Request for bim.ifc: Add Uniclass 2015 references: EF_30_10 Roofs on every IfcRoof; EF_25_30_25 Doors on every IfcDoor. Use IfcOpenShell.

First a look at what the model holds.

```python
import ifcopenshell

model = ifcopenshell.open("bim.ifc")
print(model.schema)
print("classifications:", [c.Name for c in model.by_type("IfcClassification")])
for ifc_class in ("IfcDoor", "IfcRoof", "IfcStair", "IfcWall", "IfcWindow"):
    print(ifc_class, len(model.by_type(ifc_class)))
```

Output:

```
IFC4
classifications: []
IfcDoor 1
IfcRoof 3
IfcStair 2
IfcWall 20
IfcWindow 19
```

```python
import ifcopenshell
import ifcopenshell.api.classification

model = ifcopenshell.open("bim.ifc")

system = ifcopenshell.api.classification.add_classification(model, classification="Uniclass 2015")

codes = {
    "IfcRoof": ("EF_30_10", "Roofs"),
    "IfcDoor": ("EF_25_30_25", "Doors"),
}
for ifc_class, (code, name) in codes.items():
    products = model.by_type(ifc_class)
    ifcopenshell.api.classification.add_reference(
        model, products=products, classification=system, identification=code, name=name
    )
    print(code, len(products))

model.write("bim-out.ifc")
```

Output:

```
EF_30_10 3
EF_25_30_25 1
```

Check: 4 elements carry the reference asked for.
